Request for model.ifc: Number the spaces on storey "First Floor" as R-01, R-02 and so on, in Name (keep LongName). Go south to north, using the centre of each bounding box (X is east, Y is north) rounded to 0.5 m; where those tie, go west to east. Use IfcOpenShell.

First a look at what the model holds.

```python
import ifcopenshell
import ifcopenshell.util.element
import ifcopenshell.util.placement

model = ifcopenshell.open("model.ifc")
print(model.schema)
storey = next(s for s in model.by_type("IfcBuildingStorey") if s.Name == "First Floor")
spaces = [e for e in ifcopenshell.util.element.get_decomposition(storey) if e.is_a("IfcSpace")]
for e in sorted(spaces, key=lambda e: e.id()):
    origin = ifcopenshell.util.placement.get_local_placement(e.ObjectPlacement)[:3, 3]
    print(e.id(), e.Name, e.LongName, origin.round(2) + 0.0, sep=" | ")
```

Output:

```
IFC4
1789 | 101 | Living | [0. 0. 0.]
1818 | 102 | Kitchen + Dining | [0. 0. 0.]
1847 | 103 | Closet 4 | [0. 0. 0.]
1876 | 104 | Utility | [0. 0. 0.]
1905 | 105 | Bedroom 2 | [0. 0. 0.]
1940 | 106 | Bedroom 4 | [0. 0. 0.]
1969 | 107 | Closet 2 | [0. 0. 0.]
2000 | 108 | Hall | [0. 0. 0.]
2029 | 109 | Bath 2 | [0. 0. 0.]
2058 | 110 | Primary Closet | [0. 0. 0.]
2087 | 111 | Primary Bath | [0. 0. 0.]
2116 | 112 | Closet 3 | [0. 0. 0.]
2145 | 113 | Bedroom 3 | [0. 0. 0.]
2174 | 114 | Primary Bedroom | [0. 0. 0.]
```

```python
import ifcopenshell
import ifcopenshell.geom
import ifcopenshell.util.element
import ifcopenshell.util.shape

model = ifcopenshell.open("model.ifc")
settings = ifcopenshell.geom.settings()
settings.set("use-world-coords", True)


def centre(element):
    shape = ifcopenshell.geom.create_shape(settings, element)
    return ifcopenshell.util.shape.get_bbox_centroid(shape.geometry)


storey = next(s for s in model.by_type("IfcBuildingStorey") if s.Name == "First Floor")
spaces = [e for e in ifcopenshell.util.element.get_decomposition(storey) if e.is_a("IfcSpace")]

# Insertion points can sit at a corner or the storey origin, so sort by the geometry (in metres).
centres = {e: centre(e) for e in spaces}
spaces.sort(key=lambda e: (round(centres[e][1] / 0.5), centres[e][0]))

for i, e in enumerate(spaces, start=1):
    number = f"R-{i:02d}"
    e.Name = number
    print(e.id(), number)

model.write("model_v2.ifc")
```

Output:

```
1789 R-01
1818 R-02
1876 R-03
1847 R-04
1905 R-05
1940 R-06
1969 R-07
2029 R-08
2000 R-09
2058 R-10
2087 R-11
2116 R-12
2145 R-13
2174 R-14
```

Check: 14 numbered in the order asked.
